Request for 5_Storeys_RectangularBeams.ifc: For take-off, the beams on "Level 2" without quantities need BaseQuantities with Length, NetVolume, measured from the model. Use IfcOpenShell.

First a look at what the model holds.

```python
import ifcopenshell
import ifcopenshell.util.element
import ifcopenshell.util.unit

model = ifcopenshell.open("5_Storeys_RectangularBeams.ifc")
print(model.schema)
for unit_type in ("LENGTHUNIT", "AREAUNIT", "VOLUMEUNIT"):
    print(unit_type, ifcopenshell.util.unit.calculate_unit_scale(model, unit_type))
storey = next(s for s in model.by_type("IfcBuildingStorey") if s.Name == "Level 2")
beams = [e for e in ifcopenshell.util.element.get_decomposition(storey) if e.is_a("IfcBeam")]
for e in sorted(beams, key=lambda e: e.id()):
    print(e.id(), e.is_a(), e.Name, list(ifcopenshell.util.element.get_psets(e, qtos_only=True)), sep=" | ")
```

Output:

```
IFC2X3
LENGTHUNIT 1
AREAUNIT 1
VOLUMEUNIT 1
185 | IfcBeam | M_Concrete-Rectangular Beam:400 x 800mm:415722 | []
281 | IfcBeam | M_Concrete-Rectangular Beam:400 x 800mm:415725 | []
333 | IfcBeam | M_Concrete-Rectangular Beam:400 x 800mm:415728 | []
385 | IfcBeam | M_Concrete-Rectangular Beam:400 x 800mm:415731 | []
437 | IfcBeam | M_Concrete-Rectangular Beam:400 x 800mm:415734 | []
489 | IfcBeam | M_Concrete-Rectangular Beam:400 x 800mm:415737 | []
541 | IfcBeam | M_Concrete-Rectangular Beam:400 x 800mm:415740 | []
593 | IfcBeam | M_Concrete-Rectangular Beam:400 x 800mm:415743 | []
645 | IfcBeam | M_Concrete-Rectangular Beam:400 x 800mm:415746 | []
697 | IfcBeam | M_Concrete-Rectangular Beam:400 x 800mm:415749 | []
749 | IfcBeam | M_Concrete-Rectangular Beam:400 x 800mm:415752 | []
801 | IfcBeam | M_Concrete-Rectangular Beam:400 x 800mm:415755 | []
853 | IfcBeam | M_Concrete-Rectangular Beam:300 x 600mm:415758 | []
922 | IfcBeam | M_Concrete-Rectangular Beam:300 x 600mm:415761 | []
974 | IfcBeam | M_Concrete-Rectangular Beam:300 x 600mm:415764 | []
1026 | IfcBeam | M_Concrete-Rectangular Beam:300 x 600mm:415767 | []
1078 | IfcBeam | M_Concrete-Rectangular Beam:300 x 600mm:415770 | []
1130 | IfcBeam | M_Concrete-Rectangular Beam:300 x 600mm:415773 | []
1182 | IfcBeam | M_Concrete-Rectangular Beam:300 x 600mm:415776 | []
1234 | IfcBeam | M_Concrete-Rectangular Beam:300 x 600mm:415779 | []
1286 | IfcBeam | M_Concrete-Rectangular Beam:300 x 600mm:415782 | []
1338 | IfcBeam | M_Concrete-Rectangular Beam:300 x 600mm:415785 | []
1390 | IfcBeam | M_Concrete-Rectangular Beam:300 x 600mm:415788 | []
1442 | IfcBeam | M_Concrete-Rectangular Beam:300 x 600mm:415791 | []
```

```python
import ifcopenshell
import ifcopenshell.api.pset
import ifcopenshell.geom
import ifcopenshell.util.element
import ifcopenshell.util.shape
import ifcopenshell.util.unit

model = ifcopenshell.open("5_Storeys_RectangularBeams.ifc")
unit_scale = ifcopenshell.util.unit.calculate_unit_scale(model)
volume_scale = ifcopenshell.util.unit.calculate_unit_scale(model, "VOLUMEUNIT")
settings = ifcopenshell.geom.settings()

storey = next(s for s in model.by_type("IfcBuildingStorey") if s.Name == "Level 2")
beams = [e for e in ifcopenshell.util.element.get_decomposition(storey) if e.is_a("IfcBeam")]

for e in sorted(beams, key=lambda e: e.id()):
    if ifcopenshell.util.element.get_psets(e, qtos_only=True, should_inherit=False):
        continue
    # Geometry comes back in metres, in the element's own axes.
    shape = ifcopenshell.geom.create_shape(settings, e)
    values = {
        "Length": ifcopenshell.util.shape.get_max_xyz(shape.geometry) / unit_scale,
        "NetVolume": ifcopenshell.util.shape.get_volume(shape.geometry) / volume_scale,
    }
    qto = ifcopenshell.api.pset.add_qto(model, product=e, name="BaseQuantities")
    ifcopenshell.api.pset.edit_qto(model, qto=qto, properties=values)
    print(e.id(), {k: round(v, 3) for k, v in values.items()})

model.write("5_Storeys_RectangularBeams-out.ifc")
```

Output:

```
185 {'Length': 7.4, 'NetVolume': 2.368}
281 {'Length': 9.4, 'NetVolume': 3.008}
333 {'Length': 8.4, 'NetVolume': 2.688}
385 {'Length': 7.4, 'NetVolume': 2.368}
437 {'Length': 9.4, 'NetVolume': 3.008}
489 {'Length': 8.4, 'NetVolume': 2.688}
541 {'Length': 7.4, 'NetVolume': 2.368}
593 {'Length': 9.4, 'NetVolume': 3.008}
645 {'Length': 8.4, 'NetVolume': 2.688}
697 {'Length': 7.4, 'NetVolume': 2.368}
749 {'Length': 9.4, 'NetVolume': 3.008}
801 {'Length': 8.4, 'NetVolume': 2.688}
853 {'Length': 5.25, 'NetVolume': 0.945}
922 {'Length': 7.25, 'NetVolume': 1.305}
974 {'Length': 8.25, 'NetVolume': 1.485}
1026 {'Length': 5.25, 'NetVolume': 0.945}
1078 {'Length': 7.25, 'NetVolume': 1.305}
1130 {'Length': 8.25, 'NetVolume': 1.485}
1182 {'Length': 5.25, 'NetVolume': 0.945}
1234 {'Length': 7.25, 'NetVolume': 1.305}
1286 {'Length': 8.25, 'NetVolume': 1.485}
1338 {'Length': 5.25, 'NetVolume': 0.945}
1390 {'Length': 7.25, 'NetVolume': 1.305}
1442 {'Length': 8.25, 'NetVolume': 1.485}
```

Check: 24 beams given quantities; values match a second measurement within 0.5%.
